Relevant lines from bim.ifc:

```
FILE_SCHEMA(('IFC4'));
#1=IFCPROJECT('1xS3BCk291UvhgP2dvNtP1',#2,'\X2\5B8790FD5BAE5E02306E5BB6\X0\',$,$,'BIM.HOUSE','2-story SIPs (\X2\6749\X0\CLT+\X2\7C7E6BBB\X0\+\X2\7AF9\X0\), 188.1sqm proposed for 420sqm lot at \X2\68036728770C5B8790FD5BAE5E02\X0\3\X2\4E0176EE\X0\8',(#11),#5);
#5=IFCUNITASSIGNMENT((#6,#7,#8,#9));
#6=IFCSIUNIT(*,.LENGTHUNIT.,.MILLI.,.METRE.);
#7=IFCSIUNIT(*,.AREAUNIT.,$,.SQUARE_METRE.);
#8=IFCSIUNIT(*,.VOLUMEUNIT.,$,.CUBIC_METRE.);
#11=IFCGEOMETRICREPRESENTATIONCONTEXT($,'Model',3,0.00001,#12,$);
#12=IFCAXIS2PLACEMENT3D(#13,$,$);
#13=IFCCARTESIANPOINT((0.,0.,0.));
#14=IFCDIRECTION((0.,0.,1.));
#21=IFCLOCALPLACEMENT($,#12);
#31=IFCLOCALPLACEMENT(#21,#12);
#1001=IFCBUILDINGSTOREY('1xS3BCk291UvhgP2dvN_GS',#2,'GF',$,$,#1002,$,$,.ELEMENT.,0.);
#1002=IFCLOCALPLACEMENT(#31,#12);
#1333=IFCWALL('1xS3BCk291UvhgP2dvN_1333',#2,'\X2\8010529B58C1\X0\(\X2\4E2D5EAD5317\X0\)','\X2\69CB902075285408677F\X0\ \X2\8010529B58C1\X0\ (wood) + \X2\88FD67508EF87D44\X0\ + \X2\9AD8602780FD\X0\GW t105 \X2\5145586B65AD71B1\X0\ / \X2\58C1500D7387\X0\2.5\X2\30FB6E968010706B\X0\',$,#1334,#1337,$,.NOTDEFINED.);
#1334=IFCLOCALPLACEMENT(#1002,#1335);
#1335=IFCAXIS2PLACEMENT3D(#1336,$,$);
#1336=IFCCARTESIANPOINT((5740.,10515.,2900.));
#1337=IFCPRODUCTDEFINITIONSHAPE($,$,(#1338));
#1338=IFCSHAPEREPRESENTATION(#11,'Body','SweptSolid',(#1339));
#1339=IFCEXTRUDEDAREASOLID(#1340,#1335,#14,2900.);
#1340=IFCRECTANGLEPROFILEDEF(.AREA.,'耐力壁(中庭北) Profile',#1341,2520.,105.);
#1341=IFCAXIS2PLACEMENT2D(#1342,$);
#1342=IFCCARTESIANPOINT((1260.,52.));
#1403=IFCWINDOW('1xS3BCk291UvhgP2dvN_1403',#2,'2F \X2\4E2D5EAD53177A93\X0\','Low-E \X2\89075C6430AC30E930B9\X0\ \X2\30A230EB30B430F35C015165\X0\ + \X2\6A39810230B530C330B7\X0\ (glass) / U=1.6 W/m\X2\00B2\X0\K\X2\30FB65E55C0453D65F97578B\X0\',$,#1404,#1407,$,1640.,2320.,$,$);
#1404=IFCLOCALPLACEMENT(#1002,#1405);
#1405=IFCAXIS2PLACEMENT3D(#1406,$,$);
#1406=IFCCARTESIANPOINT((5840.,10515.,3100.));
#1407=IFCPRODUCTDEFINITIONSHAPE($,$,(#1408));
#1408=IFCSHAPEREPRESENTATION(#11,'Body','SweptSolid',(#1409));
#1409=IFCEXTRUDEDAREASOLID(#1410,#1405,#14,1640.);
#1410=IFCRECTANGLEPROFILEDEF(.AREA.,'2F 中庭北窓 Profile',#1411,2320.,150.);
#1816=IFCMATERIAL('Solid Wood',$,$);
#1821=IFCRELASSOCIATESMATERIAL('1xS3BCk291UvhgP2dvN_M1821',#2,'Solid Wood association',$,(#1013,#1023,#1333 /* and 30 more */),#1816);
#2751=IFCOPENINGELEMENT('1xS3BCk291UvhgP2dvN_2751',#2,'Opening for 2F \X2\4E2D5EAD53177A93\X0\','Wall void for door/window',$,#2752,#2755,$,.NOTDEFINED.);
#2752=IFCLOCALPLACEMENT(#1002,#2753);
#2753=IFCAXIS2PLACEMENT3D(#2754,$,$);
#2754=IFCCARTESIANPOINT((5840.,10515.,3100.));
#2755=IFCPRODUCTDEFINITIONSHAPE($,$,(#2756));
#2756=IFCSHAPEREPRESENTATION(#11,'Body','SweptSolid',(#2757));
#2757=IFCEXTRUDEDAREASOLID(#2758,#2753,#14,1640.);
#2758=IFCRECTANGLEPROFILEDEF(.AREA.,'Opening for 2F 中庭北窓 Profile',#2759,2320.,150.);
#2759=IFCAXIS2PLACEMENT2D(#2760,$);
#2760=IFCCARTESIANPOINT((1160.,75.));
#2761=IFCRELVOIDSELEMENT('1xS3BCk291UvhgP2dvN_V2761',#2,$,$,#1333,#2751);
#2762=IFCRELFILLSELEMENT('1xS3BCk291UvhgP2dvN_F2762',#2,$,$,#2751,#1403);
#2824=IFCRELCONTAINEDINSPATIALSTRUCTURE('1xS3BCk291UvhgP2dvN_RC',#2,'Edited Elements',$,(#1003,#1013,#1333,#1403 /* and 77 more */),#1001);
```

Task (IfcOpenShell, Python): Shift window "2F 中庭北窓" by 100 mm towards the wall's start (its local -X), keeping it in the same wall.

```python
import ifcopenshell
import ifcopenshell.api.geometry
import ifcopenshell.util.placement

model = ifcopenshell.open("bim.ifc")

window = model.by_guid("1xS3BCk291UvhgP2dvN_1403")
opening = window.FillsVoids[0].RelatingOpeningElement
wall = opening.VoidsElements[0].RelatingBuildingElement

wall_matrix = ifcopenshell.util.placement.get_local_placement(wall.ObjectPlacement)
shift = wall_matrix[:3, 0] * -100.0
before = ifcopenshell.util.placement.get_local_placement(window.ObjectPlacement)[:3, 3].copy()

# The window is not placed relative to its opening, so move both.
for product in (opening, window):
    matrix = ifcopenshell.util.placement.get_local_placement(product.ObjectPlacement)
    matrix[:3, 3] += shift
    ifcopenshell.api.geometry.edit_object_placement(model, product=product, matrix=matrix, is_si=False)

after = ifcopenshell.util.placement.get_local_placement(window.ObjectPlacement)[:3, 3]
print("window moved by", (after - before).round(3) + 0.0)

model.write("bim_rev.ifc")
```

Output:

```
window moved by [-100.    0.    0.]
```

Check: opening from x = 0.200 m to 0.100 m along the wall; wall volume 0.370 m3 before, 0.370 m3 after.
